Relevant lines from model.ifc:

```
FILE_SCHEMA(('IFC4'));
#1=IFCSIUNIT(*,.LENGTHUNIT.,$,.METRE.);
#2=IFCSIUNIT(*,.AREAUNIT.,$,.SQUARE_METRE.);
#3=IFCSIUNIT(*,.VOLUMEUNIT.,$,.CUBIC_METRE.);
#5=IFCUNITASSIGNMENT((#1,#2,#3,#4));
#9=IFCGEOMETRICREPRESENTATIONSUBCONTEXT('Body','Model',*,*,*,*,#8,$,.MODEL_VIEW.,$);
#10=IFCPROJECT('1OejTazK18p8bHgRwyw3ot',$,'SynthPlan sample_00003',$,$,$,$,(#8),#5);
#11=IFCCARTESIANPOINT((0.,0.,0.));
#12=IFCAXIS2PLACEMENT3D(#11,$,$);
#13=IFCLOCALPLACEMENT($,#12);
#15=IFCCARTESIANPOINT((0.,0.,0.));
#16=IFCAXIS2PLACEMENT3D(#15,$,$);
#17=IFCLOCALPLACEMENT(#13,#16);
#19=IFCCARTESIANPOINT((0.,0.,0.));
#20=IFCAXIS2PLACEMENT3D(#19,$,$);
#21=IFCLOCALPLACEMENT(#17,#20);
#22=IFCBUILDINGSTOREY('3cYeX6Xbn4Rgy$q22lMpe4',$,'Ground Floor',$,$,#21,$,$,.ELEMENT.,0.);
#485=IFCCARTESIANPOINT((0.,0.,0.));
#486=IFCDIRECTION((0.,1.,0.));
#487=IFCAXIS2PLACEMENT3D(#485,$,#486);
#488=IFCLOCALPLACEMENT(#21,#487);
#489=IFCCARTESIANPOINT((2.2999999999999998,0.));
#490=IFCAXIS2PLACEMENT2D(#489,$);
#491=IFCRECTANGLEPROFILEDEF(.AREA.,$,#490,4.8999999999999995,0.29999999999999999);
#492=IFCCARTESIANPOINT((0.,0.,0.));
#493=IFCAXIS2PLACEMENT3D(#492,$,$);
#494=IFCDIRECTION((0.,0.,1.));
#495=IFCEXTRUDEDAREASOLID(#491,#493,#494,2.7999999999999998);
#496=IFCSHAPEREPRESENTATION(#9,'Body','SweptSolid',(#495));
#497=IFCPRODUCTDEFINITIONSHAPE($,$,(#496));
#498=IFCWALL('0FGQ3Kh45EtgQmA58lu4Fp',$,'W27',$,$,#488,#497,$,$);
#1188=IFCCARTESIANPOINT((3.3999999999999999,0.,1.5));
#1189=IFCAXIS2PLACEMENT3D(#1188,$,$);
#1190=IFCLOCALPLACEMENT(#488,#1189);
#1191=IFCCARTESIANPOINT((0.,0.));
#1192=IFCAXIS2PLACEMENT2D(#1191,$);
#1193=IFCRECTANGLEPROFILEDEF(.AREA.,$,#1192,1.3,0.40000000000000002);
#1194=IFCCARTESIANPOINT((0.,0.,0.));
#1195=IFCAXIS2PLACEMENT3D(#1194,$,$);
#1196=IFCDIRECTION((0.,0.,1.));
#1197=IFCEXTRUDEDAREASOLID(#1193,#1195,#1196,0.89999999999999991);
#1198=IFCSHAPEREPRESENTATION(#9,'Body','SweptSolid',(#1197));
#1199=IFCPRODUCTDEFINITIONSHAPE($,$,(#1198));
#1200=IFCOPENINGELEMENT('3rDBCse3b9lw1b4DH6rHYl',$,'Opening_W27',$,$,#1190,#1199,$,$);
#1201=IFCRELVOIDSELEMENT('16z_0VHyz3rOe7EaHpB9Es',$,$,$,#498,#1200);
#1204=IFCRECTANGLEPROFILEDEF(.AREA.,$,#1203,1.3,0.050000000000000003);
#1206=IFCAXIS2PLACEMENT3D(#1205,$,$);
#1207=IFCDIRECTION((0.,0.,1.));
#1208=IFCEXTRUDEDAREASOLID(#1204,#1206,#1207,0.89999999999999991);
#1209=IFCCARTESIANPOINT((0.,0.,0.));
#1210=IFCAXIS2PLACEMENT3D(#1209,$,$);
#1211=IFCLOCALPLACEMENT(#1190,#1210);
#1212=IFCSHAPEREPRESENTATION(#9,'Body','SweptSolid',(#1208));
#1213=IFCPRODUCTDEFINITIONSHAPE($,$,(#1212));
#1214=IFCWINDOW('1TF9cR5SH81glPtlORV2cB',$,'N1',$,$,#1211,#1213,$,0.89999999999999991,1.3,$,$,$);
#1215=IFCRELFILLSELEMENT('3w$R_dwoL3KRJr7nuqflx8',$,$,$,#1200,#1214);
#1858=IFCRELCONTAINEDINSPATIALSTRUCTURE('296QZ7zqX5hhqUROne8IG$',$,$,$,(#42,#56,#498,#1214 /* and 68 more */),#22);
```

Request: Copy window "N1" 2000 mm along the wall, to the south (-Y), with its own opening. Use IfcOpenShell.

```python
import ifcopenshell
import ifcopenshell.api.feature
import ifcopenshell.api.geometry
import ifcopenshell.api.root
import ifcopenshell.geom
import ifcopenshell.util.element
import ifcopenshell.util.placement
import ifcopenshell.util.shape

model = ifcopenshell.open("model.ifc")
settings = ifcopenshell.geom.settings()


def volume(element):
    """Net volume in cubic metres, openings subtracted."""
    shape = ifcopenshell.geom.create_shape(settings, element)
    return ifcopenshell.util.shape.get_volume(shape.geometry)


window = model.by_guid("1TF9cR5SH81glPtlORV2cB")
opening = window.FillsVoids[0].RelatingOpeningElement
wall = opening.VoidsElements[0].RelatingBuildingElement
before = volume(wall)
shift = ifcopenshell.util.placement.get_local_placement(wall.ObjectPlacement)[:3, 0] * -2.0

# copy_class copies the void relationship, type, container and properties, but no geometry.
new_opening = ifcopenshell.api.root.copy_class(model, product=opening)
new_opening.Representation = ifcopenshell.util.element.copy_deep(
    model, opening.Representation, exclude=["IfcGeometricRepresentationContext", "IfcRepresentationMap"]
)
new_window = ifcopenshell.api.root.copy_class(model, product=window)
new_window.Representation = ifcopenshell.util.element.copy_deep(
    model, window.Representation, exclude=["IfcGeometricRepresentationContext", "IfcRepresentationMap"]
)
ifcopenshell.api.feature.add_filling(model, opening=new_opening, element=new_window)

for old, new in ((opening, new_opening), (window, new_window)):
    matrix = ifcopenshell.util.placement.get_local_placement(old.ObjectPlacement)
    matrix[:3, 3] += shift
    ifcopenshell.api.geometry.edit_object_placement(model, product=new, matrix=matrix, is_si=False)

after = volume(wall)

print(f"wall volume {before:.3f} -> {after:.3f} m3")

model.write("model_edited.ifc")
```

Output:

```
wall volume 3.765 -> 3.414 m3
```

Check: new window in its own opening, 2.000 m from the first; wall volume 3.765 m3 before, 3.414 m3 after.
